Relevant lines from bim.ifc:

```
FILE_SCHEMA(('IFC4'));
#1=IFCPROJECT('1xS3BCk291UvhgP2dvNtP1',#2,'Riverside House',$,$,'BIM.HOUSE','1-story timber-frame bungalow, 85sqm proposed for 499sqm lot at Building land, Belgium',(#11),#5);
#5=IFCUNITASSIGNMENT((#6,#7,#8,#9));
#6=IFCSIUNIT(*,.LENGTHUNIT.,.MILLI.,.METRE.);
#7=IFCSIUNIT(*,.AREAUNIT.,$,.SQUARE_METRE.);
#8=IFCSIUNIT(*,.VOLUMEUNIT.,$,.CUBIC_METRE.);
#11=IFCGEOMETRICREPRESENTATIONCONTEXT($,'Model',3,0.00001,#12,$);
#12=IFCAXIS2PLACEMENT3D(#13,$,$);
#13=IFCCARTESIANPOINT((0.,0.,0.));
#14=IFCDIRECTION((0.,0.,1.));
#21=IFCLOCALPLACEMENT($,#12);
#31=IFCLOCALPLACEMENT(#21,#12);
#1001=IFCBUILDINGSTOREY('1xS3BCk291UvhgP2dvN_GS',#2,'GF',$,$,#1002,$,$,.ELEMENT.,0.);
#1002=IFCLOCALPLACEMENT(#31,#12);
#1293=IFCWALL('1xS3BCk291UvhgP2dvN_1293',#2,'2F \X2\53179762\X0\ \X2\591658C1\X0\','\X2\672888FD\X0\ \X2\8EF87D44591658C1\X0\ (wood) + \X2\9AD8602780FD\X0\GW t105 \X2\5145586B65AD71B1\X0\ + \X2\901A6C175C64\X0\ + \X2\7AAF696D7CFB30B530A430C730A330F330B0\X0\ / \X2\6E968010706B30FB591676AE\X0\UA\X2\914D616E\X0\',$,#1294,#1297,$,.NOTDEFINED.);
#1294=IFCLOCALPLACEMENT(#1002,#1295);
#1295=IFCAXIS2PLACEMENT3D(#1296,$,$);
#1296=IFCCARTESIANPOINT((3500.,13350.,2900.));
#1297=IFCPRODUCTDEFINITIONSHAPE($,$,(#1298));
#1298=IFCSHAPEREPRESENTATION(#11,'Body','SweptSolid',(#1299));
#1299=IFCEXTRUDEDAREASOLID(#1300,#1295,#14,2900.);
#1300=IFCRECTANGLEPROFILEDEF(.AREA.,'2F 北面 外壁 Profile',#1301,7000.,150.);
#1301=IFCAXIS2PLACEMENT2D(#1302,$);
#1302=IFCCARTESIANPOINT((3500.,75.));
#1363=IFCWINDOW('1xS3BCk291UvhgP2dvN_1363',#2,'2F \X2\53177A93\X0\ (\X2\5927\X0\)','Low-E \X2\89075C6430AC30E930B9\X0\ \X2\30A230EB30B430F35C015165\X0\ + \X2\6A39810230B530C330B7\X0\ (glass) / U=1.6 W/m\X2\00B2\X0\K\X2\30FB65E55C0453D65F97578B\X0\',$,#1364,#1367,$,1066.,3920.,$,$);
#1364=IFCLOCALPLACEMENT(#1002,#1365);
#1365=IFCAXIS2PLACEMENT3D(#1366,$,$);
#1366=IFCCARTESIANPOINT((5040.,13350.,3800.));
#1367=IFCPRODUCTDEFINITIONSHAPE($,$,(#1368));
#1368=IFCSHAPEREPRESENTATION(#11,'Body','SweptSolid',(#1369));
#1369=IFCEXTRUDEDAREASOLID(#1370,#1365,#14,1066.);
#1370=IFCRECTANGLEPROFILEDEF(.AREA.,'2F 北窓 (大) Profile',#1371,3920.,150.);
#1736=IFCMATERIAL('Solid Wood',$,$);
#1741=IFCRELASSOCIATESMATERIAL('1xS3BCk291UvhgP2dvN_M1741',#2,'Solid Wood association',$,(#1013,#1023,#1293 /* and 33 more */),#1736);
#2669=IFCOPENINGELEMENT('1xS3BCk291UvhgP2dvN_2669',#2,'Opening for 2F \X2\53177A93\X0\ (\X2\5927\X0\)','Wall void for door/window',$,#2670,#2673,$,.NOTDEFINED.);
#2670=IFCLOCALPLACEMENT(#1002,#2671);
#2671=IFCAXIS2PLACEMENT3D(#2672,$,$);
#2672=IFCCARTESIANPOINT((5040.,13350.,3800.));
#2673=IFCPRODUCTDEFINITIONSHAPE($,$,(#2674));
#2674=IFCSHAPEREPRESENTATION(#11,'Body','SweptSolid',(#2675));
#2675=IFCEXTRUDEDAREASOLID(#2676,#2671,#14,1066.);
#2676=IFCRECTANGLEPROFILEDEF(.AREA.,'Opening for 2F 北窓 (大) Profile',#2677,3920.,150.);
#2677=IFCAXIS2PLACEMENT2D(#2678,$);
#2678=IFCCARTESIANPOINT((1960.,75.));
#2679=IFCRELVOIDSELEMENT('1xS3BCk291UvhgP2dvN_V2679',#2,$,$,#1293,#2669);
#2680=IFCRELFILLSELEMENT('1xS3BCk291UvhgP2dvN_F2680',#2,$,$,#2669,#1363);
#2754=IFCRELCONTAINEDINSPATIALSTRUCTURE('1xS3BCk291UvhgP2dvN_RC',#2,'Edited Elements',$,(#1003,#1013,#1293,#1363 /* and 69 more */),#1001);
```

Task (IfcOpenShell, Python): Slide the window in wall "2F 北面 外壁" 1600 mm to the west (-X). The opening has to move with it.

```python
import ifcopenshell
import ifcopenshell.api.geometry
import ifcopenshell.util.placement

model = ifcopenshell.open("bim.ifc")

window = model.by_id(1363)
opening = window.FillsVoids[0].RelatingOpeningElement
wall = opening.VoidsElements[0].RelatingBuildingElement

wall_matrix = ifcopenshell.util.placement.get_local_placement(wall.ObjectPlacement)
shift = wall_matrix[:3, 0] * -1600.0
before = ifcopenshell.util.placement.get_local_placement(window.ObjectPlacement)[:3, 3].copy()

# The window is not placed relative to its opening, so move both.
for product in (opening, window):
    matrix = ifcopenshell.util.placement.get_local_placement(product.ObjectPlacement)
    matrix[:3, 3] += shift
    ifcopenshell.api.geometry.edit_object_placement(model, product=product, matrix=matrix, is_si=False)

after = ifcopenshell.util.placement.get_local_placement(window.ObjectPlacement)[:3, 3]
print("window moved by", (after - before).round(3) + 0.0)

model.write("bim_updated.ifc")
```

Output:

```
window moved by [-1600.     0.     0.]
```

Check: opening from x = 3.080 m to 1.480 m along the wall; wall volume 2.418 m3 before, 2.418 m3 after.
